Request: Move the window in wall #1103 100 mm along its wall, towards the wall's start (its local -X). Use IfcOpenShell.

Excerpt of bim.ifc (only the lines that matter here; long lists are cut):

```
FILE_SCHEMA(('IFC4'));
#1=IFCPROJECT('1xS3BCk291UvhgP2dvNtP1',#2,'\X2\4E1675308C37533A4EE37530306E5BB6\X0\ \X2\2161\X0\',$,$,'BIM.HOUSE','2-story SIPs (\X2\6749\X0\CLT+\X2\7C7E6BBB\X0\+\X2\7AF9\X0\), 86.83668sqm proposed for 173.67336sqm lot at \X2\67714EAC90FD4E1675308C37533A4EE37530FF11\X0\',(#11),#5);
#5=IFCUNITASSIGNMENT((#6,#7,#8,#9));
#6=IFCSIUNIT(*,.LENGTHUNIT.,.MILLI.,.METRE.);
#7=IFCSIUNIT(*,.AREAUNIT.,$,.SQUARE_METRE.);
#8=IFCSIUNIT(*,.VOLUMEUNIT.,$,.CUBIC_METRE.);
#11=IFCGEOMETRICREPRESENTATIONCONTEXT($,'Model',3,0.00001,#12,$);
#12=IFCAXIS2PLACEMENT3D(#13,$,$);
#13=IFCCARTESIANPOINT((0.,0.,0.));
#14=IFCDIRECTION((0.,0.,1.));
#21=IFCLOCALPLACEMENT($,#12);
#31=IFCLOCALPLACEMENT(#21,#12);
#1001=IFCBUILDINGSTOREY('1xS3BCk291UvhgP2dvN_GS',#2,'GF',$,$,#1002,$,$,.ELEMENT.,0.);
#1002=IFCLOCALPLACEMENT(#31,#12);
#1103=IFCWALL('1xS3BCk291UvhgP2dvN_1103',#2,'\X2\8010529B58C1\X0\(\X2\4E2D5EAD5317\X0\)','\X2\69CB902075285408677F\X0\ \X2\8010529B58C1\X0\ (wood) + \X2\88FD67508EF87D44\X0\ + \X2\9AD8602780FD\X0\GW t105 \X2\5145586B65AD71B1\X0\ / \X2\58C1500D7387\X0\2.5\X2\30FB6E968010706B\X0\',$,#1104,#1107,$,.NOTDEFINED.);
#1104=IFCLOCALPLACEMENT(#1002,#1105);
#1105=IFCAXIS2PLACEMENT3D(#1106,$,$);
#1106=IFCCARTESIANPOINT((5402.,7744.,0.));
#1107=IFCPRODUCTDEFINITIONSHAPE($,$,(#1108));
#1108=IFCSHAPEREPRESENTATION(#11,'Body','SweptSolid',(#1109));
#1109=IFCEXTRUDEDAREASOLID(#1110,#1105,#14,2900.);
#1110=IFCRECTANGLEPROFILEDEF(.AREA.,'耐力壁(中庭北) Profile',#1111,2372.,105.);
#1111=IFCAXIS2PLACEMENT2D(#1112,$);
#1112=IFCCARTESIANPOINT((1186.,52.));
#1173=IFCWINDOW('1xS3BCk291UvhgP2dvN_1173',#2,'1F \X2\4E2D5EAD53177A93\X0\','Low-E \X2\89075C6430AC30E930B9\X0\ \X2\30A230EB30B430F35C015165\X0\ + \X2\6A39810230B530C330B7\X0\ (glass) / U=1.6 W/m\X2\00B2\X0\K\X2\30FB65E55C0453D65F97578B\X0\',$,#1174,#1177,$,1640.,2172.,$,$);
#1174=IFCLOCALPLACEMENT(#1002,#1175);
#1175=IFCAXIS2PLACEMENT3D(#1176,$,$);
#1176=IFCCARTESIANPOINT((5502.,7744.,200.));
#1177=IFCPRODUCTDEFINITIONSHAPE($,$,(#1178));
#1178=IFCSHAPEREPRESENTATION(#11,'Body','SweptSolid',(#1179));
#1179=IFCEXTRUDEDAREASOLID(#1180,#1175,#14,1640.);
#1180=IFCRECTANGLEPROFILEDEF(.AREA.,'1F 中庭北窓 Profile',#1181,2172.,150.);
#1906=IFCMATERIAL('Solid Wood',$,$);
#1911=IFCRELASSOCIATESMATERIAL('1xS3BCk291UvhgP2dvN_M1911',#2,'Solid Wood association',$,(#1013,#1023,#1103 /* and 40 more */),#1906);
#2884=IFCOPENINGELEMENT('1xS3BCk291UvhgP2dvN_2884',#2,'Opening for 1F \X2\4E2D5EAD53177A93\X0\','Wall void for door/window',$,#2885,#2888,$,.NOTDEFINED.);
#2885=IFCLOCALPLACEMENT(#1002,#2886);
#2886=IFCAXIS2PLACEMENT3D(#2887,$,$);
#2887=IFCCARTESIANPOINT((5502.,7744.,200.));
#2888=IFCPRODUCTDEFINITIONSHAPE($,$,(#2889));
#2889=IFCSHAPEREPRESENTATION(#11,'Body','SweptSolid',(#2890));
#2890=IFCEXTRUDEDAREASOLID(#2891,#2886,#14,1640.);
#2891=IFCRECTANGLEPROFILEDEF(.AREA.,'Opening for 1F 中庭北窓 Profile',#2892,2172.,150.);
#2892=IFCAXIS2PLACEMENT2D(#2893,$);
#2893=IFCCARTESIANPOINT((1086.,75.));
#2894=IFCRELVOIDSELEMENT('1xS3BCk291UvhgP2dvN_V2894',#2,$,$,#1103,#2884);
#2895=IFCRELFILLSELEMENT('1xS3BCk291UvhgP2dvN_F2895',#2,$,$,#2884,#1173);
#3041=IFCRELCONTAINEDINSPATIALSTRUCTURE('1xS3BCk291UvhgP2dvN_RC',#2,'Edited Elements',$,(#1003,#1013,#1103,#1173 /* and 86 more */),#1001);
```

```python
import ifcopenshell
import ifcopenshell.api.geometry
import ifcopenshell.util.placement

model = ifcopenshell.open("bim.ifc")

window = model.by_guid("1xS3BCk291UvhgP2dvN_1173")
opening = window.FillsVoids[0].RelatingOpeningElement
wall = opening.VoidsElements[0].RelatingBuildingElement

wall_matrix = ifcopenshell.util.placement.get_local_placement(wall.ObjectPlacement)
shift = wall_matrix[:3, 0] * -100.0
before = ifcopenshell.util.placement.get_local_placement(window.ObjectPlacement)[:3, 3].copy()

# The window is not placed relative to its opening, so move both.
for product in (opening, window):
    matrix = ifcopenshell.util.placement.get_local_placement(product.ObjectPlacement)
    matrix[:3, 3] += shift
    ifcopenshell.api.geometry.edit_object_placement(model, product=product, matrix=matrix, is_si=False)

after = ifcopenshell.util.placement.get_local_placement(window.ObjectPlacement)[:3, 3]
print("window moved by", (after - before).round(3) + 0.0)

model.write("bim_v2.ifc")
```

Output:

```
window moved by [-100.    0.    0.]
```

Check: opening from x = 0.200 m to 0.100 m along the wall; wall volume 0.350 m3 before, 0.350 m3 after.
